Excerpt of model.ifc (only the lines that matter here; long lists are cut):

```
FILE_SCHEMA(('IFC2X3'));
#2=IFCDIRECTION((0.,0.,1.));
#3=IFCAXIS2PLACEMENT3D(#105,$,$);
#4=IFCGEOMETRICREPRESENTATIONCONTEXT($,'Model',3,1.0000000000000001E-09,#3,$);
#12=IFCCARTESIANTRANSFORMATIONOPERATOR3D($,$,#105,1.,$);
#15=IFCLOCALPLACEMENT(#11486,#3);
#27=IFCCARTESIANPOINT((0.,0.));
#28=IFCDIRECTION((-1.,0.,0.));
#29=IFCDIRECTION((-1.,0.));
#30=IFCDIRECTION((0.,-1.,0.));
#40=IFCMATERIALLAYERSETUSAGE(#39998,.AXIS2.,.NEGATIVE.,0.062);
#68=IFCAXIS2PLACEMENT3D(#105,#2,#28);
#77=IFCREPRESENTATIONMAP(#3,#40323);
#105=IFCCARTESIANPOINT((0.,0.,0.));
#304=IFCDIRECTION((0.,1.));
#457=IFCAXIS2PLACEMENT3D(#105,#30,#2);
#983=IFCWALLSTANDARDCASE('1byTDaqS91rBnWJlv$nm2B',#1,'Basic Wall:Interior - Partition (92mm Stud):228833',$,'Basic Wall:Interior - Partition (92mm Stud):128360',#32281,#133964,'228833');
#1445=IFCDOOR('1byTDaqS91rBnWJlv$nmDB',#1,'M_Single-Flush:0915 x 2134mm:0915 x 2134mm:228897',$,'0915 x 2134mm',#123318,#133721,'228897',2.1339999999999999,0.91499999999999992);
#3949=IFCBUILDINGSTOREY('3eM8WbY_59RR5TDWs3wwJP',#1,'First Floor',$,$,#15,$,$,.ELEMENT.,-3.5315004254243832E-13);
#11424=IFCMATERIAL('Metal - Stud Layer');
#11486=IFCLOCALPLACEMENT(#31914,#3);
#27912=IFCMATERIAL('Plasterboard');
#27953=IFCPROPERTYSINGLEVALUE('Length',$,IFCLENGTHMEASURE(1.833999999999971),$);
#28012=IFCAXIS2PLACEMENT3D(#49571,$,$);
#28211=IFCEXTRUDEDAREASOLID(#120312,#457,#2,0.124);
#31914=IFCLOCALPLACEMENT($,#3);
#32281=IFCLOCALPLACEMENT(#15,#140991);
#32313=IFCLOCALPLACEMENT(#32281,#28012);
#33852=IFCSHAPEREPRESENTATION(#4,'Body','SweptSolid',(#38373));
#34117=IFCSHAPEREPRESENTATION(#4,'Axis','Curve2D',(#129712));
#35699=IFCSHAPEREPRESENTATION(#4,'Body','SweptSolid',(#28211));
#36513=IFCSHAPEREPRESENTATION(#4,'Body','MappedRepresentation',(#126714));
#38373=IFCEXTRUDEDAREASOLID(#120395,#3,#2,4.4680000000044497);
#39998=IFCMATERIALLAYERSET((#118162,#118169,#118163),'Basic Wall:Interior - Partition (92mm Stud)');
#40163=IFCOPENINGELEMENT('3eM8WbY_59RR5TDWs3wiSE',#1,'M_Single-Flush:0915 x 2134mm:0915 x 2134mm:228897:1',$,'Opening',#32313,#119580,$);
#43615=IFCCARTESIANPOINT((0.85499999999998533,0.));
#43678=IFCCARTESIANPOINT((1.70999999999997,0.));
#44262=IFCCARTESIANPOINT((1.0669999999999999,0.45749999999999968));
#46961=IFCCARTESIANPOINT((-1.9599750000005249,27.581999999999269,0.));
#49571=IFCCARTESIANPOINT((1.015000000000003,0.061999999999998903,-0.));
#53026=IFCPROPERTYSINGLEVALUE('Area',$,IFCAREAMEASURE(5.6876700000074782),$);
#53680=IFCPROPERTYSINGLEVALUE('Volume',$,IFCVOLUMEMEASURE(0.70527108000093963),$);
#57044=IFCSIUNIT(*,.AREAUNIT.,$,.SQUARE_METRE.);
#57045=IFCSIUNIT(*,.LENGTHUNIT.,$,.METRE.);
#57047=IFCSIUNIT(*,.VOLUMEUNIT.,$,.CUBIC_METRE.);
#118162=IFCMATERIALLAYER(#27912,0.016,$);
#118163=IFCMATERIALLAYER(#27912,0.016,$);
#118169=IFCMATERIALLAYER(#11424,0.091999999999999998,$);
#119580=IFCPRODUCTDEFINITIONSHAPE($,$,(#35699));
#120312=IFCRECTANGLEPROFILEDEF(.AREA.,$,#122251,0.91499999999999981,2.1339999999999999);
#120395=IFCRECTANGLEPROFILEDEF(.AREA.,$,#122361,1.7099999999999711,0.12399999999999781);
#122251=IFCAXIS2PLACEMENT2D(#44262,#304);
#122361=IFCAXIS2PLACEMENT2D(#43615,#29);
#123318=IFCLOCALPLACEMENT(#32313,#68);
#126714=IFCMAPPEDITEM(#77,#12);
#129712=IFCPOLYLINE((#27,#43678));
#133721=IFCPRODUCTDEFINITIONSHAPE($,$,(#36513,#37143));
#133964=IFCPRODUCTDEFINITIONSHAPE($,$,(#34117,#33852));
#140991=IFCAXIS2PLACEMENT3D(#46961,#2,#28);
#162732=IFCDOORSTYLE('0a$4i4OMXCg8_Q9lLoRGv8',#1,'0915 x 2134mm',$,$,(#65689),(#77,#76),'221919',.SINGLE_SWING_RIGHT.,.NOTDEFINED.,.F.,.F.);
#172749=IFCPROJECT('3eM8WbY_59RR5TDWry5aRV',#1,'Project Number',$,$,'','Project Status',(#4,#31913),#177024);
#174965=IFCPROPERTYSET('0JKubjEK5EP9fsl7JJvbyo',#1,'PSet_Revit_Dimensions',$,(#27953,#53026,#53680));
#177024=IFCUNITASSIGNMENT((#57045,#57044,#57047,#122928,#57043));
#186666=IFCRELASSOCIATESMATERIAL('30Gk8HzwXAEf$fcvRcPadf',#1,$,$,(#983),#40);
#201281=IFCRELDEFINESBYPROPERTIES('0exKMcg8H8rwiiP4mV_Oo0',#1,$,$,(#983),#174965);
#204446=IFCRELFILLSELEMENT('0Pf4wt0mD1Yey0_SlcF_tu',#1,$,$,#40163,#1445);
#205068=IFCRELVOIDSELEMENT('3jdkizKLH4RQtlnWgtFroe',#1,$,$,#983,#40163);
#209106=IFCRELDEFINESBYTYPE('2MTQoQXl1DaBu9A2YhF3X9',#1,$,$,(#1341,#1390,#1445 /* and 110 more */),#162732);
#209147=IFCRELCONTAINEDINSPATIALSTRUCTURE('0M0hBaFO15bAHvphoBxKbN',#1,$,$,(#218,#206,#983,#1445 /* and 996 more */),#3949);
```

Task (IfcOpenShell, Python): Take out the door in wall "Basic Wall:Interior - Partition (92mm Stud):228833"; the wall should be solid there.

```python
import ifcopenshell
import ifcopenshell.api.feature
import ifcopenshell.api.pset
import ifcopenshell.api.root
import ifcopenshell.geom
import ifcopenshell.util.element
import ifcopenshell.util.shape
import ifcopenshell.util.unit

model = ifcopenshell.open("model.ifc")
area_scale = ifcopenshell.util.unit.calculate_unit_scale(model, "AREAUNIT")
volume_scale = ifcopenshell.util.unit.calculate_unit_scale(model, "VOLUMEUNIT")
settings = ifcopenshell.geom.settings()


def volume(element):
    """Net volume in cubic metres, openings subtracted."""
    shape = ifcopenshell.geom.create_shape(settings, element)
    return ifcopenshell.util.shape.get_volume(shape.geometry)


door = model.by_guid("1byTDaqS91rBnWJlv$nmDB")
opening = door.FillsVoids[0].RelatingOpeningElement
wall = opening.VoidsElements[0].RelatingBuildingElement
before = volume(wall)

ifcopenshell.api.root.remove_product(model, product=door)
ifcopenshell.api.feature.remove_feature(model, feature=opening)

after = volume(wall)
thickness = 0.124  # wall thickness in metres

# Update the wall's stored quantities.
pset = model.by_id(ifcopenshell.util.element.get_pset(wall, "PSet_Revit_Dimensions", should_inherit=False)["id"])
ifcopenshell.api.pset.edit_pset(model, pset=pset, properties={
    "Area": model.create_entity("IfcAreaMeasure", after / thickness / area_scale),
    "Volume": model.create_entity("IfcVolumeMeasure", after / volume_scale),
})

print(f"wall volume {before:.3f} -> {after:.3f} m3")

model.write("model_rev.ifc")
```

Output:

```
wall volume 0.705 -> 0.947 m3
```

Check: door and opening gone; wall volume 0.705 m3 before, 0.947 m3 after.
